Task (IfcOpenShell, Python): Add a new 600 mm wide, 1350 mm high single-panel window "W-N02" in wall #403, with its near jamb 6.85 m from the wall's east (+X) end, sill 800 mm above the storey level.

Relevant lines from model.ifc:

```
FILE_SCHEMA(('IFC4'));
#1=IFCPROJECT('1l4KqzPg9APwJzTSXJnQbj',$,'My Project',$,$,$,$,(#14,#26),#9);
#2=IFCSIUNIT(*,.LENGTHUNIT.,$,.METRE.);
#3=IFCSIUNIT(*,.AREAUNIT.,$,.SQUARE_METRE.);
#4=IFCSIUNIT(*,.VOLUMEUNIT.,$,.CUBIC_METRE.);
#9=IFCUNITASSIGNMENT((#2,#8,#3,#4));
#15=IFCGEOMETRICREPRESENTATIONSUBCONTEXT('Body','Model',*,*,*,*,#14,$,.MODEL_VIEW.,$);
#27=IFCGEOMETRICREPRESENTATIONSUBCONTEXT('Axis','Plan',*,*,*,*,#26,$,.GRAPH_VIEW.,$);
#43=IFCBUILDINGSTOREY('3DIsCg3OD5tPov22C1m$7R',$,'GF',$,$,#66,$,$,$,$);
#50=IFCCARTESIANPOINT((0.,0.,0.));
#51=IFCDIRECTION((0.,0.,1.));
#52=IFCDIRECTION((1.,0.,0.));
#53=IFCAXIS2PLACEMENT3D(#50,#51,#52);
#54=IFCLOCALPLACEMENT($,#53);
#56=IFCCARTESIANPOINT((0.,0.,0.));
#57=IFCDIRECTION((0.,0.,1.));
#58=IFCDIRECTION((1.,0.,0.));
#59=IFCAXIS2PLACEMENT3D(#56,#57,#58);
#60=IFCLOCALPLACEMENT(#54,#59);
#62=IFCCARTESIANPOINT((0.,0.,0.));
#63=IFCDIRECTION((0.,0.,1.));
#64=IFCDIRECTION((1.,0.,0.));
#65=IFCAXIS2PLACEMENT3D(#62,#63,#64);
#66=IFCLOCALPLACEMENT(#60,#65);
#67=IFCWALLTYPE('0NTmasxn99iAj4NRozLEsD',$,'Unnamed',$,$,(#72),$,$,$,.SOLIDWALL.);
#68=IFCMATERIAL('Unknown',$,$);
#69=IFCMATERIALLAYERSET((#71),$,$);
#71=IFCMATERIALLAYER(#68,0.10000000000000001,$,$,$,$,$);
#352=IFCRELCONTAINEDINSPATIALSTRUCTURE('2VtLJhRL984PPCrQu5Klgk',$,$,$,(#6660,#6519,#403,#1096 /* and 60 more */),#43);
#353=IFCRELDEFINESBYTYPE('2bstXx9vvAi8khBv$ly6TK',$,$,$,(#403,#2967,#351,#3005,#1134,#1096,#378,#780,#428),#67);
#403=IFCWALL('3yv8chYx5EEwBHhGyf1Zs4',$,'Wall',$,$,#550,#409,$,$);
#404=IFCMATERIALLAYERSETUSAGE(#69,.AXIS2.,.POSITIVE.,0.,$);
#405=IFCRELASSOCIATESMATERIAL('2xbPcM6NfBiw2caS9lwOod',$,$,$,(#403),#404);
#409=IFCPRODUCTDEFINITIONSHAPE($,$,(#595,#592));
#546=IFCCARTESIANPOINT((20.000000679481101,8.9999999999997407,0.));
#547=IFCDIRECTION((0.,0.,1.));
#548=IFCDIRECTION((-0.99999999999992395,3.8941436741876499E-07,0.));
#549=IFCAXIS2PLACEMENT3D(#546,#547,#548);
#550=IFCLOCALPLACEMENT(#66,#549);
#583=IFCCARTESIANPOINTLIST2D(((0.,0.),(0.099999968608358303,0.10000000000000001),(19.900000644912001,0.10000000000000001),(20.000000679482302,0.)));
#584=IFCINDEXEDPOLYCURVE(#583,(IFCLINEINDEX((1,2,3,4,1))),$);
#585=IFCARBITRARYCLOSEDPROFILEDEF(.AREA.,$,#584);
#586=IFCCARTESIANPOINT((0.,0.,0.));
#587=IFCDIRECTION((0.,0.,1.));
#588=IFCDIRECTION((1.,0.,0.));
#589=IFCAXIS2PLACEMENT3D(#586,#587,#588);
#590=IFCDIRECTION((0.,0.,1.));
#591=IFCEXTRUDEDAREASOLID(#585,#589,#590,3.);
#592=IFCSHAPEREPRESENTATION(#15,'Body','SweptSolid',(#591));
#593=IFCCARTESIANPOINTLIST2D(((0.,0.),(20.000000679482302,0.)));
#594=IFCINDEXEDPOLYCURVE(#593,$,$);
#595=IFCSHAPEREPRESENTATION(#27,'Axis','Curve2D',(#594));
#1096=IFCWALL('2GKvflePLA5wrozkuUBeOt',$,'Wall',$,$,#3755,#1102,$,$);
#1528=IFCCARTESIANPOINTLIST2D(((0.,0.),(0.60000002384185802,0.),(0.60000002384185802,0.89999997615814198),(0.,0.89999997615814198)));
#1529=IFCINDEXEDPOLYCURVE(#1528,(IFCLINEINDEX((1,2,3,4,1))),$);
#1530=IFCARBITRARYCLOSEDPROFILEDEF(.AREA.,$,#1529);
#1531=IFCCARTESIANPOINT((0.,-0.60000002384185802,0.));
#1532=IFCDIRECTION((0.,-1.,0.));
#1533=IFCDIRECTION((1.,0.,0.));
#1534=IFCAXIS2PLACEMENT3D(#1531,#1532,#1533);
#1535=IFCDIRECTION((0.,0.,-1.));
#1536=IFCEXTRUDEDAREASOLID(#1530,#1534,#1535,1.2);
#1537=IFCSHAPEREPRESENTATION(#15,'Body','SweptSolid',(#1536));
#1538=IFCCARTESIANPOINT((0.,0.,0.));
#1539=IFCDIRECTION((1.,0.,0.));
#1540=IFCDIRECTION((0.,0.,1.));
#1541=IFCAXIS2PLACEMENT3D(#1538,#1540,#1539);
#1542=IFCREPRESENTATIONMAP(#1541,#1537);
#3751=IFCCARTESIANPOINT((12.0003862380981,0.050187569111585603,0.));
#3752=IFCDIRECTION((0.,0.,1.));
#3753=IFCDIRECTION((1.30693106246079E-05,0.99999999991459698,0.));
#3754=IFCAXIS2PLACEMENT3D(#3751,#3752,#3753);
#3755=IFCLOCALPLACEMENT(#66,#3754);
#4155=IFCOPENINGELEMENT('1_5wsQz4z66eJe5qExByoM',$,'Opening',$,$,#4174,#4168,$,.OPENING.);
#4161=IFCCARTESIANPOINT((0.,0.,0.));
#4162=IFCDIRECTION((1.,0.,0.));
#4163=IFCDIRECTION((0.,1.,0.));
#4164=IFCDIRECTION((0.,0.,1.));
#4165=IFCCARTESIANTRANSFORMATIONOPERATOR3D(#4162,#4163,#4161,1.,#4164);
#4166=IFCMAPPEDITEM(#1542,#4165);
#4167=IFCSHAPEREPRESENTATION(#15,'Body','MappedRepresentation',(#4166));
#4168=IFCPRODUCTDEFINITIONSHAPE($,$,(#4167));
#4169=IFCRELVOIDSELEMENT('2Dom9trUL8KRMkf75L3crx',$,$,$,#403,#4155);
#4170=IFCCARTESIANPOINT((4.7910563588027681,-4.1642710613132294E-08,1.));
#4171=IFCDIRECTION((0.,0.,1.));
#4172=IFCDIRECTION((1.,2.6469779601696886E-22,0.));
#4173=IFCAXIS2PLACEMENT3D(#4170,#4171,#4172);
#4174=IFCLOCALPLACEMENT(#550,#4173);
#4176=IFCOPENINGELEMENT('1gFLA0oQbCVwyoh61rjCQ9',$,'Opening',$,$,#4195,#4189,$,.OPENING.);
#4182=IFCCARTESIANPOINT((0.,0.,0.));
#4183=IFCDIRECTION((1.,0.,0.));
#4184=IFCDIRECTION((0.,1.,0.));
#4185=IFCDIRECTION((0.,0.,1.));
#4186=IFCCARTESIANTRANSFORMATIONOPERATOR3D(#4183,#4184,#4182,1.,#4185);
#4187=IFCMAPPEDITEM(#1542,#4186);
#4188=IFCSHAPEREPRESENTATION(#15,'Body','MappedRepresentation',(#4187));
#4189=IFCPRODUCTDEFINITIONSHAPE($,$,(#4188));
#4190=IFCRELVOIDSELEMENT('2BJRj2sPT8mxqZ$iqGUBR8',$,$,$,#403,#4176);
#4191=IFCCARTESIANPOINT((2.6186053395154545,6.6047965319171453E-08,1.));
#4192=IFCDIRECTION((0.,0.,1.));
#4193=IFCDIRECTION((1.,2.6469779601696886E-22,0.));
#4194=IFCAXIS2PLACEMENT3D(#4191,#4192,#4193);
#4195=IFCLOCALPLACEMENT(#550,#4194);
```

```python
import numpy as np
import ifcopenshell
import ifcopenshell.api.feature
import ifcopenshell.api.geometry
import ifcopenshell.api.root
import ifcopenshell.api.spatial
import ifcopenshell.geom
import ifcopenshell.util.element
import ifcopenshell.util.placement
import ifcopenshell.util.representation
import ifcopenshell.util.shape
import ifcopenshell.util.unit

model = ifcopenshell.open("model.ifc")
unit_scale = ifcopenshell.util.unit.calculate_unit_scale(model)
settings = ifcopenshell.geom.settings()


def volume(element):
    """Net volume in cubic metres, openings subtracted."""
    shape = ifcopenshell.geom.create_shape(settings, element)
    return ifcopenshell.util.shape.get_volume(shape.geometry)


wall = model.by_guid("3yv8chYx5EEwBHhGyf1Zs4")
storey = ifcopenshell.util.element.get_container(wall, ifc_class="IfcBuildingStorey")
context = ifcopenshell.util.representation.get_context(model, "Model", "Body", "MODEL_VIEW")
before = volume(wall)

width, height, from_end, sill = 0.6, 1.35, 6.85, 0.8  # metres

# The wall runs along its own X axis, and the end named is its -X end.
wall_shape = ifcopenshell.geom.create_shape(settings, wall)
x, y, z = ifcopenshell.util.shape.get_vertices(wall_shape.geometry).T
start = x.min() + from_end
face, thickness = float(y.min()), float(y.max() - y.min())
wall_matrix = ifcopenshell.util.placement.get_local_placement(wall.ObjectPlacement)
level = ifcopenshell.util.placement.get_local_placement(storey.ObjectPlacement)[2, 3]


def in_wall(x, y):
    """Placement at x, y metres in the wall's axes, at sill height."""
    matrix = wall_matrix.copy()
    matrix[:, 3] = wall_matrix @ np.array([x / unit_scale, y / unit_scale, 0.0, 1.0])
    matrix[2, 3] = level + sill / unit_scale
    return matrix


# Opening: a box that overshoots both wall faces by 50 mm.
opening = ifcopenshell.api.root.create_entity(model, ifc_class="IfcOpeningElement", predefined_type="OPENING")
box = ifcopenshell.api.geometry.add_wall_representation(
    model, context=context, length=width, height=height, thickness=thickness + 0.1
)
ifcopenshell.api.geometry.assign_representation(model, product=opening, representation=box)
ifcopenshell.api.geometry.edit_object_placement(model, product=opening, matrix=in_wall(start, face - 0.05), is_si=False)
ifcopenshell.api.feature.add_feature(model, feature=opening, element=wall)

window = ifcopenshell.api.root.create_entity(model, ifc_class="IfcWindow", name="W-N02", predefined_type="WINDOW")
window.OverallWidth, window.OverallHeight = width / unit_scale, height / unit_scale
window.PartitioningType = "SINGLE_PANEL"
body = ifcopenshell.api.geometry.add_window_representation(
    model,
    context=context,
    overall_width=window.OverallWidth,
    overall_height=window.OverallHeight,
    partition_type="SINGLE_PANEL",
)
ifcopenshell.api.geometry.assign_representation(model, product=window, representation=body)
ifcopenshell.api.spatial.assign_container(model, products=[window], relating_structure=storey)
ifcopenshell.api.feature.add_filling(model, opening=opening, element=window)

# Centre the window in the wall's thickness.
ifcopenshell.api.geometry.edit_object_placement(model, product=window, matrix=in_wall(start, face), is_si=False)
window_shape = ifcopenshell.geom.create_shape(settings, window)
depth = ifcopenshell.util.shape.get_vertices(window_shape.geometry)[:, 1]
offset = face + thickness / 2 - (depth.min() + depth.max()) / 2
ifcopenshell.api.geometry.edit_object_placement(model, product=window, matrix=in_wall(start, offset), is_si=False)

after = volume(wall)

print(f"wall volume {before:.3f} -> {after:.3f} m3")

model.write("model_rev.ifc")
```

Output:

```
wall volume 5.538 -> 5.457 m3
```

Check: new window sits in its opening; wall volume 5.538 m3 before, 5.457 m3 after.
